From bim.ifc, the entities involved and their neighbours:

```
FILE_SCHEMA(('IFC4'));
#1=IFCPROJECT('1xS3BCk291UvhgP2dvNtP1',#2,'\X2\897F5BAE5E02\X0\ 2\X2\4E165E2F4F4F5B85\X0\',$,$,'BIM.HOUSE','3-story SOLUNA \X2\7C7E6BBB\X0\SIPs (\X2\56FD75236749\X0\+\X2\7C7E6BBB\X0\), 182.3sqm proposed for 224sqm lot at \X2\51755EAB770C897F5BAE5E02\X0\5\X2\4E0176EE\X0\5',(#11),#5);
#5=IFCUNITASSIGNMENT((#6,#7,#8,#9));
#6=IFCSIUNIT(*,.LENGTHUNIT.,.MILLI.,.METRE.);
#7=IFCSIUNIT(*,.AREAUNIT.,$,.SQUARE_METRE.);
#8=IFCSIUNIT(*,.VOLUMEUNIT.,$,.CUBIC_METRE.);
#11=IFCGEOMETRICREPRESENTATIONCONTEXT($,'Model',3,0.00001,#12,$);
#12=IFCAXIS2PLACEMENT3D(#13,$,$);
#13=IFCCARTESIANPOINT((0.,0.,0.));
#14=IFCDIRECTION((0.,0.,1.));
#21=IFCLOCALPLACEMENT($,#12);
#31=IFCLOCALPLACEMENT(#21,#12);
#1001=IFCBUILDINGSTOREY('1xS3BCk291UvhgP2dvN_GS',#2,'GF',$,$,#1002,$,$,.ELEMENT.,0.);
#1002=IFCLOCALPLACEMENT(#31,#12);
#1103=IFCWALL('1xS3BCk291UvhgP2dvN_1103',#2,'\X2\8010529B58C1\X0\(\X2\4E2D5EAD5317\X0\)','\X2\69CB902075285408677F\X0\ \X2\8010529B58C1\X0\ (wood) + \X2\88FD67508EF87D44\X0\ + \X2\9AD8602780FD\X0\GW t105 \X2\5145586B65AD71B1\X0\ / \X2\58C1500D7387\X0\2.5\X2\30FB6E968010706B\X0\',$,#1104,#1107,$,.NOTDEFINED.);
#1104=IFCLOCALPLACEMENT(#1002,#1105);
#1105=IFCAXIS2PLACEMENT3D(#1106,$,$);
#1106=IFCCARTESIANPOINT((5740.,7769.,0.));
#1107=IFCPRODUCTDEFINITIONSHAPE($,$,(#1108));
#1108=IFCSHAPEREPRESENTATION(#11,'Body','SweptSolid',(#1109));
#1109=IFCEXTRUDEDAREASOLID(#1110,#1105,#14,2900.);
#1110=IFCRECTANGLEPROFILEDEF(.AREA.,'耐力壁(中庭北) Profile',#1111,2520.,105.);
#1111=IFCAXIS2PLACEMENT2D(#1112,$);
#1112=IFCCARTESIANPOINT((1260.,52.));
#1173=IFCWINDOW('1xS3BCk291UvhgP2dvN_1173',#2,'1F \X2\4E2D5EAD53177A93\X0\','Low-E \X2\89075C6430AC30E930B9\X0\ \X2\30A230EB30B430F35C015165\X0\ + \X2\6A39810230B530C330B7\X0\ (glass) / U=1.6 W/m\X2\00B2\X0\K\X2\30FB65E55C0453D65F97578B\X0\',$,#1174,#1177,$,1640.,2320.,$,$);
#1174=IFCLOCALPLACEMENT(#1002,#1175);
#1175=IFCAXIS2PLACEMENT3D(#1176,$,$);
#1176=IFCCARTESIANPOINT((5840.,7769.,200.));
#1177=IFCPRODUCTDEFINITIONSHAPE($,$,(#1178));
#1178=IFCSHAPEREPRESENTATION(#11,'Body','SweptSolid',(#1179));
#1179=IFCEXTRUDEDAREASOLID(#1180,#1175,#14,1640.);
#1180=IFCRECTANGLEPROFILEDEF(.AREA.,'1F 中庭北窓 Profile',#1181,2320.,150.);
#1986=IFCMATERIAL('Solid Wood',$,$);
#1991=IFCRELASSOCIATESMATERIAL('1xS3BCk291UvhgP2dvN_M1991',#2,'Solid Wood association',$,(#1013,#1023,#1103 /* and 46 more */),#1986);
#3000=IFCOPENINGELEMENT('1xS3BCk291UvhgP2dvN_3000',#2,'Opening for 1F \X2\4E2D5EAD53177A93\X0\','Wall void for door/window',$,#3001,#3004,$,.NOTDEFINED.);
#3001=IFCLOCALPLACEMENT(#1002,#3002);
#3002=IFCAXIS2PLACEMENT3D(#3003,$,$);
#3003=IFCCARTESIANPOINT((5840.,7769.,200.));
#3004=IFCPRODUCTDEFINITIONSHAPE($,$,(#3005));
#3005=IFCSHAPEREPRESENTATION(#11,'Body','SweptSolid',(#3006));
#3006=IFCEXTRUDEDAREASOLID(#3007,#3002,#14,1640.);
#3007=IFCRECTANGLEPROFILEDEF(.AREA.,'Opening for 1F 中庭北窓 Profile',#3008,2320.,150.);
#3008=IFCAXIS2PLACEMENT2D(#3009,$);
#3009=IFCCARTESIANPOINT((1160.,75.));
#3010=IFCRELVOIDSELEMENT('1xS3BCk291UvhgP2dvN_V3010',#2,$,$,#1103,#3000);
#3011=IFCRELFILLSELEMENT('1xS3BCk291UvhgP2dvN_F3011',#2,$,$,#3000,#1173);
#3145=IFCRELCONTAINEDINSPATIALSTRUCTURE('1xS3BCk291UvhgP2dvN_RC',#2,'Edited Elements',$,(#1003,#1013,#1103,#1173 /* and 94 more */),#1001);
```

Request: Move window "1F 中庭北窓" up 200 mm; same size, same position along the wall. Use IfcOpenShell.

```python
import numpy as np
import ifcopenshell
import ifcopenshell.api.geometry
import ifcopenshell.util.placement
import ifcopenshell.util.unit

model = ifcopenshell.open("bim.ifc")
unit_scale = ifcopenshell.util.unit.calculate_unit_scale(model)

window = model.by_guid("1xS3BCk291UvhgP2dvN_1173")
opening = window.FillsVoids[0].RelatingOpeningElement
dz = 200.0

shift = np.array([0.0, 0.0, dz])
# The window is not placed relative to its opening, so move both.
for product in (opening, window):
    matrix = ifcopenshell.util.placement.get_local_placement(product.ObjectPlacement)
    matrix[:3, 3] += shift
    ifcopenshell.api.geometry.edit_object_placement(model, product=product, matrix=matrix, is_si=False)

print(f"moved by {dz * unit_scale:+.3f} m")

model.write("bim_v2.ifc")
```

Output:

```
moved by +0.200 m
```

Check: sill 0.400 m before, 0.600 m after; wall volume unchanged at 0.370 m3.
